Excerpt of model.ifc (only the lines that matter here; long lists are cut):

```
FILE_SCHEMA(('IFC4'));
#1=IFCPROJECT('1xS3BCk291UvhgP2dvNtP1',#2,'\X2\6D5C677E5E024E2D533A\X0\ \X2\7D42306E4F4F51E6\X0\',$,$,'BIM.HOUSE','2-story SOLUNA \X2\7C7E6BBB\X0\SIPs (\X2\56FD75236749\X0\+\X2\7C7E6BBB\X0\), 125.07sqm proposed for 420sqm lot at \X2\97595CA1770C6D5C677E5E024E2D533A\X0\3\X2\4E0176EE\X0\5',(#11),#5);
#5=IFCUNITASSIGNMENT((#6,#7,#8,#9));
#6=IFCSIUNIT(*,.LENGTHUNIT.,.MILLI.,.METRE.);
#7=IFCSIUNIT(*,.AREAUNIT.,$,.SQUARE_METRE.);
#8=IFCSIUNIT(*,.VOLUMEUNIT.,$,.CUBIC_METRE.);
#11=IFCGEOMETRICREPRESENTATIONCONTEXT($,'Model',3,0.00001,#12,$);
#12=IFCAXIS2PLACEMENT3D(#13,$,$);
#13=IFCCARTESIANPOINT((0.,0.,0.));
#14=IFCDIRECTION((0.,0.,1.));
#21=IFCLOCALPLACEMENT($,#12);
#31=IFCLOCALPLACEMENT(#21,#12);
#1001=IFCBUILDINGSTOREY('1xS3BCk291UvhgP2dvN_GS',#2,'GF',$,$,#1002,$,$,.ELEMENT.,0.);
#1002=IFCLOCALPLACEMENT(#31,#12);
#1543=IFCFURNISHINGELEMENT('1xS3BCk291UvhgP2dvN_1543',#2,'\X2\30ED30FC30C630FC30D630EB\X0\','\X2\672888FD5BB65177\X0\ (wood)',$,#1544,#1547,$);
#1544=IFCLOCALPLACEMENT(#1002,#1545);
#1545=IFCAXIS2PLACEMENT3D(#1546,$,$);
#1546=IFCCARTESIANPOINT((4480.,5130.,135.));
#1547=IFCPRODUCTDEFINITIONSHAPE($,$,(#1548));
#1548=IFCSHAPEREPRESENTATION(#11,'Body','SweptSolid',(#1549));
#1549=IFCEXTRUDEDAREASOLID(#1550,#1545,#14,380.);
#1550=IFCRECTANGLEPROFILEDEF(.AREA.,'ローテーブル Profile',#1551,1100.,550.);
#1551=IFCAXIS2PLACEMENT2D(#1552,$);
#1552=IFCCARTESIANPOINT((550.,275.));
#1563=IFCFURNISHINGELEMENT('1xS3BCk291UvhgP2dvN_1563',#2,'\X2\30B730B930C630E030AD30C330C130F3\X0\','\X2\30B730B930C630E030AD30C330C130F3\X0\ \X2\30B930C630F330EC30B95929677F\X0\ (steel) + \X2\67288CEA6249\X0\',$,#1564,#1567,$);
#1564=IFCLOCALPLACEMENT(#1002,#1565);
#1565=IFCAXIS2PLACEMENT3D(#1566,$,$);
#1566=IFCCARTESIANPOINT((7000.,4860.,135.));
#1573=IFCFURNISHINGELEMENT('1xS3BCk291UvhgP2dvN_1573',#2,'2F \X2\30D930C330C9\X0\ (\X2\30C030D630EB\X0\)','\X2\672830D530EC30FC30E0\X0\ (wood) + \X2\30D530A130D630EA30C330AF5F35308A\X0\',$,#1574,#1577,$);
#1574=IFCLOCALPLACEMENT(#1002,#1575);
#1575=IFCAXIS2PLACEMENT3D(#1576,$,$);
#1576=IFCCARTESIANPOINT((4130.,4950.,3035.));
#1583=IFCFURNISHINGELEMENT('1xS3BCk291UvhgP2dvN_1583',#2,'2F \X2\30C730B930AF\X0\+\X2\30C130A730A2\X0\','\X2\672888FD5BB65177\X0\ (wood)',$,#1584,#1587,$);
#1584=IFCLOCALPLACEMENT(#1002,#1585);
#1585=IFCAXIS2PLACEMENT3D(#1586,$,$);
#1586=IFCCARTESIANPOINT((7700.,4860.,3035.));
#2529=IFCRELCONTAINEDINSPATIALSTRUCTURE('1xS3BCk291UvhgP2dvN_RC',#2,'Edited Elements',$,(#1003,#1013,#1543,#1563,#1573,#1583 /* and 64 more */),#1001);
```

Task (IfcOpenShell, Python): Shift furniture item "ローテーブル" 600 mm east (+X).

```python
import ifcopenshell
import ifcopenshell.api.geometry
import ifcopenshell.util.placement

model = ifcopenshell.open("model.ifc")

item = model.by_guid("1xS3BCk291UvhgP2dvN_1543")
matrix = ifcopenshell.util.placement.get_local_placement(item.ObjectPlacement)
matrix[0, 3] += 600.0
ifcopenshell.api.geometry.edit_object_placement(model, product=item, matrix=matrix, is_si=False)

print(ifcopenshell.util.placement.get_local_placement(item.ObjectPlacement).round(3) + 0.0)

model.write("model_v2.ifc")
```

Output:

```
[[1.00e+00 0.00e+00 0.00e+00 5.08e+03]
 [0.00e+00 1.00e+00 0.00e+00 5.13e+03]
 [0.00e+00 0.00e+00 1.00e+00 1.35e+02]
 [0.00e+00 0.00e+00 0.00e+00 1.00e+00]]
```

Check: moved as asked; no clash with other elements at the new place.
